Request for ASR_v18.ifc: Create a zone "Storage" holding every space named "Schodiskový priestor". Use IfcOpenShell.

First a look at what the model holds.

```python
import ifcopenshell

model = ifcopenshell.open("ASR_v18.ifc")
print(model.schema)
seen = {}
for space in model.by_type("IfcSpace"):
    seen[space.LongName] = seen.get(space.LongName, 0) + 1
for name, count in sorted(seen.items(), key=str):
    print(count, "x", name)
print("zones:", [z.Name for z in model.by_type("IfcZone")][:20])
```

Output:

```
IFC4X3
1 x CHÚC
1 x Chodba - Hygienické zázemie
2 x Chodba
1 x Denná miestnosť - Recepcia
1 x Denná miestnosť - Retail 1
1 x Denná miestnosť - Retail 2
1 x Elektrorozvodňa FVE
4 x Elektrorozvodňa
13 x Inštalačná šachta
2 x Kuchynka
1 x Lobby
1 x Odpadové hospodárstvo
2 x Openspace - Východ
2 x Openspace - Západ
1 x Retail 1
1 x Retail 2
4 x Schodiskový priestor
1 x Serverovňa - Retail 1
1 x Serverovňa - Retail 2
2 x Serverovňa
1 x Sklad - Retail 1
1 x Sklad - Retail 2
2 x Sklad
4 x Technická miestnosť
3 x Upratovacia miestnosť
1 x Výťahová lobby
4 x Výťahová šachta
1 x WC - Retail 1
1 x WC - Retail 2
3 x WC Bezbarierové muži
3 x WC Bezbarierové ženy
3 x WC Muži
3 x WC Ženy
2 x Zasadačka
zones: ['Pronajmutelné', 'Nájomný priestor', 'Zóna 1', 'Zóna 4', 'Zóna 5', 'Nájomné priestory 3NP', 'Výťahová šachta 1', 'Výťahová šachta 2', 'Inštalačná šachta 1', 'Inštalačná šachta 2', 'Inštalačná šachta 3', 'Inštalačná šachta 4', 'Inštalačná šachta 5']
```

```python
import ifcopenshell
import ifcopenshell.api.group
import ifcopenshell.api.root

model = ifcopenshell.open("ASR_v18.ifc")

names = {"Schodiskový priestor"}
spaces = [s for s in model.by_type("IfcSpace") if s.LongName in names]

zone = ifcopenshell.api.root.create_entity(model, ifc_class="IfcZone", name="Storage")
ifcopenshell.api.group.assign_group(model, products=spaces, group=zone)
print(len(spaces), "spaces in", zone.Name)

model.write("ASR_v18_updated.ifc")
```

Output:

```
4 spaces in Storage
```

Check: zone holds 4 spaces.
